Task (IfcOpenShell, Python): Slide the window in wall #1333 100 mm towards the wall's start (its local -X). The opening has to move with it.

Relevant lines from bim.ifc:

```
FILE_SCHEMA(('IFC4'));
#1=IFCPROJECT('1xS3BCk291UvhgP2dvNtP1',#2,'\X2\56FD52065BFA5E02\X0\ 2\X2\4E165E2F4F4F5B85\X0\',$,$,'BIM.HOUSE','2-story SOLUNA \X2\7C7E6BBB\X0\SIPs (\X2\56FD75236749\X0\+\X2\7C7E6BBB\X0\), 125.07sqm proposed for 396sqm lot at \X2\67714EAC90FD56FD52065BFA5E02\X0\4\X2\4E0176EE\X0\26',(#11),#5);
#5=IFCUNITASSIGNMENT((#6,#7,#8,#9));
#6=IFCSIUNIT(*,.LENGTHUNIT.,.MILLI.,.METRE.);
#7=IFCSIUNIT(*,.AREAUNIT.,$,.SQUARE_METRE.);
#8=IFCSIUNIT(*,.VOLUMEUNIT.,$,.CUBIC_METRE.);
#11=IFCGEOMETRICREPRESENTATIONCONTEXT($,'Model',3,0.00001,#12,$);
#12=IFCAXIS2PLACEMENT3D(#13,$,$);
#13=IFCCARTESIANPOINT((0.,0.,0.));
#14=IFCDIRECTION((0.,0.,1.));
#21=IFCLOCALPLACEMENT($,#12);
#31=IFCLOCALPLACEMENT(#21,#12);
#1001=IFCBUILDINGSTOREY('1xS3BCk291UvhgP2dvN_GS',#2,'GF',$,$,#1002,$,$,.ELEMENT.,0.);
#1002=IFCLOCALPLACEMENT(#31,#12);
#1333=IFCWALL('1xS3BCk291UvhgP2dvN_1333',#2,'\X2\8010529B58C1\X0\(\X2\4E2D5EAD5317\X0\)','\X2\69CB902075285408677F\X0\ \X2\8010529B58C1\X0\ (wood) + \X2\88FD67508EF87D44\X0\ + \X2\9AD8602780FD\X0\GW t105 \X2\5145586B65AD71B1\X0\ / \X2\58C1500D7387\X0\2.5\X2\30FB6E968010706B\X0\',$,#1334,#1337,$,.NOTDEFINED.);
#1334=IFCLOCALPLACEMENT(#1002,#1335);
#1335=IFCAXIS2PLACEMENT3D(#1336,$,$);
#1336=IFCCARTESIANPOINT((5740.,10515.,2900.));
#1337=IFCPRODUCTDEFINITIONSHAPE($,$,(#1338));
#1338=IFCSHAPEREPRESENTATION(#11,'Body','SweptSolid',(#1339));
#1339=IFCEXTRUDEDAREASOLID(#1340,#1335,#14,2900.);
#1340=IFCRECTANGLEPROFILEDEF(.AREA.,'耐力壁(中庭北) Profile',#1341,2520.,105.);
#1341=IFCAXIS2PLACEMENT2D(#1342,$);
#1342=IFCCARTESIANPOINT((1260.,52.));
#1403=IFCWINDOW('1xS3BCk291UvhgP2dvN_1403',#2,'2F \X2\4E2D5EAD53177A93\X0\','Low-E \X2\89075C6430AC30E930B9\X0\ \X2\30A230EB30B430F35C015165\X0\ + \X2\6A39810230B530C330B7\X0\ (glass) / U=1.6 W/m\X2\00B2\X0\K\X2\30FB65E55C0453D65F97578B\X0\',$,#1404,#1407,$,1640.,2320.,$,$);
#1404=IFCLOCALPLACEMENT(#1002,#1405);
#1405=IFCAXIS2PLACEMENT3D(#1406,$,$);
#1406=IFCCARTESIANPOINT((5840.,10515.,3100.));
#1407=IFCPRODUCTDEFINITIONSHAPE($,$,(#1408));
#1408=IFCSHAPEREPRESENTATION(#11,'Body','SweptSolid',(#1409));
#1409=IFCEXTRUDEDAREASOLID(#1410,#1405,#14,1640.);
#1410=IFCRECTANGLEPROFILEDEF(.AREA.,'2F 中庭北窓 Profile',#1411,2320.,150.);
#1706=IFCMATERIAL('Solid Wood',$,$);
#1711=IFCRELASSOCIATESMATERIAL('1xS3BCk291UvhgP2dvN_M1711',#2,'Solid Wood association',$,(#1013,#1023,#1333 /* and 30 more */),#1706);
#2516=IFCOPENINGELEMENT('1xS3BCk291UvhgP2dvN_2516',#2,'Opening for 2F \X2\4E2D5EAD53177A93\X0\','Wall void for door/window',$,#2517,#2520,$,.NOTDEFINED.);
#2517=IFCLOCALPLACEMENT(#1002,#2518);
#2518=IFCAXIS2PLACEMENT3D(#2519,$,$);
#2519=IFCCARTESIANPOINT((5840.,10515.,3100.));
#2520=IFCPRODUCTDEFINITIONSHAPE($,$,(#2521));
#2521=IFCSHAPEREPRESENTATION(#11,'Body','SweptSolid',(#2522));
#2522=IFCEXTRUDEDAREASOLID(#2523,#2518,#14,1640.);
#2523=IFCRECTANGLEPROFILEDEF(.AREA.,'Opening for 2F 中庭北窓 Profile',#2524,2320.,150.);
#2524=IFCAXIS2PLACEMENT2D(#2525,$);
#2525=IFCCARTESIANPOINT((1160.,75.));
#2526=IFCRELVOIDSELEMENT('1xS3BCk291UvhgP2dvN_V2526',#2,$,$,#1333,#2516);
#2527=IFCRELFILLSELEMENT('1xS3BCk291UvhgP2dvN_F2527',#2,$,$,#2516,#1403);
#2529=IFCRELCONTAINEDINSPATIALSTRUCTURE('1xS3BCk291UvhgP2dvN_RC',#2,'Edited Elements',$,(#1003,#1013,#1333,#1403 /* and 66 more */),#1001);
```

```python
import ifcopenshell
import ifcopenshell.api.geometry
import ifcopenshell.util.placement
import ifcopenshell.util.unit

model = ifcopenshell.open("bim.ifc")
unit_scale = ifcopenshell.util.unit.calculate_unit_scale(model)

window = model.by_guid("1xS3BCk291UvhgP2dvN_1403")
opening = window.FillsVoids[0].RelatingOpeningElement
wall = opening.VoidsElements[0].RelatingBuildingElement

wall_matrix = ifcopenshell.util.placement.get_local_placement(wall.ObjectPlacement)
shift = wall_matrix[:3, 0] * -0.1 / unit_scale
before = ifcopenshell.util.placement.get_local_placement(window.ObjectPlacement)[:3, 3].copy()

# The window is not placed relative to its opening, so move both.
for product in (opening, window):
    matrix = ifcopenshell.util.placement.get_local_placement(product.ObjectPlacement)
    matrix[:3, 3] += shift
    ifcopenshell.api.geometry.edit_object_placement(model, product=product, matrix=matrix, is_si=False)

after = ifcopenshell.util.placement.get_local_placement(window.ObjectPlacement)[:3, 3]
print("window moved by", (after - before).round(3) + 0.0)

model.write("bim-out.ifc")
```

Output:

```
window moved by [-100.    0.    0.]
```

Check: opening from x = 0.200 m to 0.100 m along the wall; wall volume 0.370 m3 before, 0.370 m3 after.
